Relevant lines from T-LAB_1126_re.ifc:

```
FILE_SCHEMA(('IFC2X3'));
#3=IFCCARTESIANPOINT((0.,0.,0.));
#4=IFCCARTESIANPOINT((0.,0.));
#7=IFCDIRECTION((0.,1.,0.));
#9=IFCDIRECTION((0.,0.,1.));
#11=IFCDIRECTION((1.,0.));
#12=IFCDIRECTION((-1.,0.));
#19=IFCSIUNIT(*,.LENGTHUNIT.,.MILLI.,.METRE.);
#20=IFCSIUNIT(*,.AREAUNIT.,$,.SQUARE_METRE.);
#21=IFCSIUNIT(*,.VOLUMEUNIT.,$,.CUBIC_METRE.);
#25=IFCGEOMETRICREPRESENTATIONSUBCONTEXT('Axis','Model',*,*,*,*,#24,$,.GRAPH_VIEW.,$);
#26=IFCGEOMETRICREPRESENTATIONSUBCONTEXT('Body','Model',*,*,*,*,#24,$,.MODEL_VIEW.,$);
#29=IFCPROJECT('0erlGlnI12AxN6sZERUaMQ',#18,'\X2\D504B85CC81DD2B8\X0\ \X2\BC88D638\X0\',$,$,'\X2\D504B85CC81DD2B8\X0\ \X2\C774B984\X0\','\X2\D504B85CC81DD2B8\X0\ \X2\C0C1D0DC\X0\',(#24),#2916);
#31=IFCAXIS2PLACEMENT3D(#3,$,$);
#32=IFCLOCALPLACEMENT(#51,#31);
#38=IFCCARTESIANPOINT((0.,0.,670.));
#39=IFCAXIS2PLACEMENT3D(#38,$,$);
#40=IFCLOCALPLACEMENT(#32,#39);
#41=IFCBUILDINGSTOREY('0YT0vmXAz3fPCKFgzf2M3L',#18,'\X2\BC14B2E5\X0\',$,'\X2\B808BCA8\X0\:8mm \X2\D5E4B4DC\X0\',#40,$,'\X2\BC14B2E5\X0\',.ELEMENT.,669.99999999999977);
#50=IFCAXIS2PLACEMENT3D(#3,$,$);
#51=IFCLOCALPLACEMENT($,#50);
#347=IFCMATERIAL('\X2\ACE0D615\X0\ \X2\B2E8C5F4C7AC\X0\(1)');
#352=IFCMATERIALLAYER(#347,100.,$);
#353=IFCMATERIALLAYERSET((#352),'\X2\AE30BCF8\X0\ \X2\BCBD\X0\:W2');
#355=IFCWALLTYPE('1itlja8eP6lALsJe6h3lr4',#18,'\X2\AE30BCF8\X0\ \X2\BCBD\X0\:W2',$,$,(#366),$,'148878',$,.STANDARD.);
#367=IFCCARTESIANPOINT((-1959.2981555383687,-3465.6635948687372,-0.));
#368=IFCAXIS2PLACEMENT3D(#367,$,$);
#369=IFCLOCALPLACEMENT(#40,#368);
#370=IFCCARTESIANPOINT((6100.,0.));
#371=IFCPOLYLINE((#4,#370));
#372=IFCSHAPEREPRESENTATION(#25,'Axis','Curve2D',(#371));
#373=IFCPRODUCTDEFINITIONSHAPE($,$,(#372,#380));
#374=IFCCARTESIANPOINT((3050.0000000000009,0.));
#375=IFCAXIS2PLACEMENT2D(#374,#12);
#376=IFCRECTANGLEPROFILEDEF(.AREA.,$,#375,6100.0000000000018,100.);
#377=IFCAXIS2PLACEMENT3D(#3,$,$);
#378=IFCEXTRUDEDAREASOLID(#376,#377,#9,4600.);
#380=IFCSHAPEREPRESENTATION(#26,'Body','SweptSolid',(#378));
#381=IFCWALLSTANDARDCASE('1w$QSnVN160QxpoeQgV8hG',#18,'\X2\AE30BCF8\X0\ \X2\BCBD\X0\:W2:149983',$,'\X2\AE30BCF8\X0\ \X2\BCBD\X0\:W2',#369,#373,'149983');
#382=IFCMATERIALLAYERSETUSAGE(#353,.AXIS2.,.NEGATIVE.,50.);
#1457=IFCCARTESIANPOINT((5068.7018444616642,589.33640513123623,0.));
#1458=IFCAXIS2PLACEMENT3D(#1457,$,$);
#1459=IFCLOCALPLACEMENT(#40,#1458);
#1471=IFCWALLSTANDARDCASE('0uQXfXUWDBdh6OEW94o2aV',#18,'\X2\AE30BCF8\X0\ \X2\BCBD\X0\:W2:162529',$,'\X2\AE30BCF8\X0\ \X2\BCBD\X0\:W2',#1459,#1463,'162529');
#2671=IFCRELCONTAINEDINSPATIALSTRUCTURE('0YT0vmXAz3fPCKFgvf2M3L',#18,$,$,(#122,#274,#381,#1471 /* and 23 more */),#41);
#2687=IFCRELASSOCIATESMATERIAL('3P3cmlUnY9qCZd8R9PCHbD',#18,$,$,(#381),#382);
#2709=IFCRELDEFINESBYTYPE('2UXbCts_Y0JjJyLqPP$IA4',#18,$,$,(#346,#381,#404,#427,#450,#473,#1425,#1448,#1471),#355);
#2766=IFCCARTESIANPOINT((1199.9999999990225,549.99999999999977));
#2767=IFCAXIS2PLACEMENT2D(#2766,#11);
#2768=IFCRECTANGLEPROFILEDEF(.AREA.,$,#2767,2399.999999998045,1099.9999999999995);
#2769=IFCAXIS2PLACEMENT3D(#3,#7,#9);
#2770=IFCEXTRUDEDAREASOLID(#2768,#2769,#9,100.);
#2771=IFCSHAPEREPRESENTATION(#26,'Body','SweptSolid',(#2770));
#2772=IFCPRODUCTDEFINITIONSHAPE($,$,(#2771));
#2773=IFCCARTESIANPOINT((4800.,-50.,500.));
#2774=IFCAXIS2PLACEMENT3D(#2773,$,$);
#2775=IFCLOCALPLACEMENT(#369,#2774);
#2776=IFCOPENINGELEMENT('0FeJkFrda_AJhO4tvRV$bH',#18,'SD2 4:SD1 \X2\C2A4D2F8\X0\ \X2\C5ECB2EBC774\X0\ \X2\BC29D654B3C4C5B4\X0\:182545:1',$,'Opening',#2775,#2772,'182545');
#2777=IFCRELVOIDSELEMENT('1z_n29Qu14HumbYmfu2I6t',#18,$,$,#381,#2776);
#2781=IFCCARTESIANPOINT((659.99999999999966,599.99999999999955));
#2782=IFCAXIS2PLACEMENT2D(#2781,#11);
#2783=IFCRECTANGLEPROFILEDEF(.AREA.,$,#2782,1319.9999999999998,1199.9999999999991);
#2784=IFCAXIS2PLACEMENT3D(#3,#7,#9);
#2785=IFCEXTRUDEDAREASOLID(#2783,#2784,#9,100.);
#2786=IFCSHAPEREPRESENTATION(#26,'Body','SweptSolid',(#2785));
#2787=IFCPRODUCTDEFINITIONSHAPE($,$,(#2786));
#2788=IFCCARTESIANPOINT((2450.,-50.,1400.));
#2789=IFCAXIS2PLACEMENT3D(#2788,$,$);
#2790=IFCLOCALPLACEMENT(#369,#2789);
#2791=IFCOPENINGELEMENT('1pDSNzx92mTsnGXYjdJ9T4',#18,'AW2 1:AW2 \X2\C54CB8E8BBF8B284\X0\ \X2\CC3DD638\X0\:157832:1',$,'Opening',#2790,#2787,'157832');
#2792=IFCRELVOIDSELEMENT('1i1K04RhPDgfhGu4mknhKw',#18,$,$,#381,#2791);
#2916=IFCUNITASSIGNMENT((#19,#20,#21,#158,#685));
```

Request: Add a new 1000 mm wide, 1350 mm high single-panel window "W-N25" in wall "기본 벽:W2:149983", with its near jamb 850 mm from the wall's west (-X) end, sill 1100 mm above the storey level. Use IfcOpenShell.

```python
import numpy as np
import ifcopenshell
import ifcopenshell.api.feature
import ifcopenshell.api.geometry
import ifcopenshell.api.root
import ifcopenshell.api.spatial
import ifcopenshell.api.type
import ifcopenshell.geom
import ifcopenshell.util.element
import ifcopenshell.util.placement
import ifcopenshell.util.representation
import ifcopenshell.util.shape
import ifcopenshell.util.unit

model = ifcopenshell.open("T-LAB_1126_re.ifc")
unit_scale = ifcopenshell.util.unit.calculate_unit_scale(model)
settings = ifcopenshell.geom.settings()


def volume(element):
    """Net volume in cubic metres, openings subtracted."""
    shape = ifcopenshell.geom.create_shape(settings, element)
    return ifcopenshell.util.shape.get_volume(shape.geometry)


wall = model.by_id(381)
storey = ifcopenshell.util.element.get_container(wall, ifc_class="IfcBuildingStorey")
context = ifcopenshell.util.representation.get_context(model, "Model", "Body", "MODEL_VIEW")
before = volume(wall)

width, height, from_end, sill = 1, 1.35, 0.85, 1.1  # metres

# The wall runs along its own X axis, and the end named is its -X end.
wall_shape = ifcopenshell.geom.create_shape(settings, wall)
x, y, z = ifcopenshell.util.shape.get_vertices(wall_shape.geometry).T
start = x.min() + from_end
face, thickness = float(y.min()), float(y.max() - y.min())
wall_matrix = ifcopenshell.util.placement.get_local_placement(wall.ObjectPlacement)
level = ifcopenshell.util.placement.get_local_placement(storey.ObjectPlacement)[2, 3]


def in_wall(x, y):
    """Placement at x, y metres in the wall's axes, at sill height."""
    matrix = wall_matrix.copy()
    matrix[:, 3] = wall_matrix @ np.array([x / unit_scale, y / unit_scale, 0.0, 1.0])
    matrix[2, 3] = level + sill / unit_scale
    return matrix


# Opening: a box that overshoots both wall faces by 50 mm.
opening = ifcopenshell.api.root.create_entity(model, ifc_class="IfcOpeningElement")
box = ifcopenshell.api.geometry.add_wall_representation(
    model, context=context, length=width, height=height, thickness=thickness + 0.1
)
ifcopenshell.api.geometry.assign_representation(model, product=opening, representation=box)
ifcopenshell.api.geometry.edit_object_placement(model, product=opening, matrix=in_wall(start, face - 0.05), is_si=False)
ifcopenshell.api.feature.add_feature(model, feature=opening, element=wall)

window = ifcopenshell.api.root.create_entity(model, ifc_class="IfcWindow", name="W-N25")
window.OverallWidth, window.OverallHeight = width / unit_scale, height / unit_scale
body = ifcopenshell.api.geometry.add_window_representation(
    model,
    context=context,
    overall_width=window.OverallWidth,
    overall_height=window.OverallHeight,
    partition_type="SINGLE_PANEL",
)
ifcopenshell.api.geometry.assign_representation(model, product=window, representation=body)
ifcopenshell.api.spatial.assign_container(model, products=[window], relating_structure=storey)
fills = ifcopenshell.api.feature.add_filling(model, opening=opening, element=window)
fills.OwnerHistory = window.OwnerHistory  # required in IFC2X3

# IFC2X3 keeps the operation on the window style.
style = ifcopenshell.api.root.create_entity(model, ifc_class="IfcWindowStyle", name="W-N25")
style.OperationType, style.ConstructionType = "SINGLE_PANEL", "NOTDEFINED"
style.ParameterTakesPrecedence = style.Sizeable = False
ifcopenshell.api.type.assign_type(model, related_objects=[window], relating_type=style)

# Centre the window in the wall's thickness.
ifcopenshell.api.geometry.edit_object_placement(model, product=window, matrix=in_wall(start, face), is_si=False)
window_shape = ifcopenshell.geom.create_shape(settings, window)
depth = ifcopenshell.util.shape.get_vertices(window_shape.geometry)[:, 1]
offset = face + thickness / 2 - (depth.min() + depth.max()) / 2
ifcopenshell.api.geometry.edit_object_placement(model, product=window, matrix=in_wall(start, offset), is_si=False)

after = volume(wall)

print(f"wall volume {before:.3f} -> {after:.3f} m3")

model.write("T-LAB_1126_re-out.ifc")
```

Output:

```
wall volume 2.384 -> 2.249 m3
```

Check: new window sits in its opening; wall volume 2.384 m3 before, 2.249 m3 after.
